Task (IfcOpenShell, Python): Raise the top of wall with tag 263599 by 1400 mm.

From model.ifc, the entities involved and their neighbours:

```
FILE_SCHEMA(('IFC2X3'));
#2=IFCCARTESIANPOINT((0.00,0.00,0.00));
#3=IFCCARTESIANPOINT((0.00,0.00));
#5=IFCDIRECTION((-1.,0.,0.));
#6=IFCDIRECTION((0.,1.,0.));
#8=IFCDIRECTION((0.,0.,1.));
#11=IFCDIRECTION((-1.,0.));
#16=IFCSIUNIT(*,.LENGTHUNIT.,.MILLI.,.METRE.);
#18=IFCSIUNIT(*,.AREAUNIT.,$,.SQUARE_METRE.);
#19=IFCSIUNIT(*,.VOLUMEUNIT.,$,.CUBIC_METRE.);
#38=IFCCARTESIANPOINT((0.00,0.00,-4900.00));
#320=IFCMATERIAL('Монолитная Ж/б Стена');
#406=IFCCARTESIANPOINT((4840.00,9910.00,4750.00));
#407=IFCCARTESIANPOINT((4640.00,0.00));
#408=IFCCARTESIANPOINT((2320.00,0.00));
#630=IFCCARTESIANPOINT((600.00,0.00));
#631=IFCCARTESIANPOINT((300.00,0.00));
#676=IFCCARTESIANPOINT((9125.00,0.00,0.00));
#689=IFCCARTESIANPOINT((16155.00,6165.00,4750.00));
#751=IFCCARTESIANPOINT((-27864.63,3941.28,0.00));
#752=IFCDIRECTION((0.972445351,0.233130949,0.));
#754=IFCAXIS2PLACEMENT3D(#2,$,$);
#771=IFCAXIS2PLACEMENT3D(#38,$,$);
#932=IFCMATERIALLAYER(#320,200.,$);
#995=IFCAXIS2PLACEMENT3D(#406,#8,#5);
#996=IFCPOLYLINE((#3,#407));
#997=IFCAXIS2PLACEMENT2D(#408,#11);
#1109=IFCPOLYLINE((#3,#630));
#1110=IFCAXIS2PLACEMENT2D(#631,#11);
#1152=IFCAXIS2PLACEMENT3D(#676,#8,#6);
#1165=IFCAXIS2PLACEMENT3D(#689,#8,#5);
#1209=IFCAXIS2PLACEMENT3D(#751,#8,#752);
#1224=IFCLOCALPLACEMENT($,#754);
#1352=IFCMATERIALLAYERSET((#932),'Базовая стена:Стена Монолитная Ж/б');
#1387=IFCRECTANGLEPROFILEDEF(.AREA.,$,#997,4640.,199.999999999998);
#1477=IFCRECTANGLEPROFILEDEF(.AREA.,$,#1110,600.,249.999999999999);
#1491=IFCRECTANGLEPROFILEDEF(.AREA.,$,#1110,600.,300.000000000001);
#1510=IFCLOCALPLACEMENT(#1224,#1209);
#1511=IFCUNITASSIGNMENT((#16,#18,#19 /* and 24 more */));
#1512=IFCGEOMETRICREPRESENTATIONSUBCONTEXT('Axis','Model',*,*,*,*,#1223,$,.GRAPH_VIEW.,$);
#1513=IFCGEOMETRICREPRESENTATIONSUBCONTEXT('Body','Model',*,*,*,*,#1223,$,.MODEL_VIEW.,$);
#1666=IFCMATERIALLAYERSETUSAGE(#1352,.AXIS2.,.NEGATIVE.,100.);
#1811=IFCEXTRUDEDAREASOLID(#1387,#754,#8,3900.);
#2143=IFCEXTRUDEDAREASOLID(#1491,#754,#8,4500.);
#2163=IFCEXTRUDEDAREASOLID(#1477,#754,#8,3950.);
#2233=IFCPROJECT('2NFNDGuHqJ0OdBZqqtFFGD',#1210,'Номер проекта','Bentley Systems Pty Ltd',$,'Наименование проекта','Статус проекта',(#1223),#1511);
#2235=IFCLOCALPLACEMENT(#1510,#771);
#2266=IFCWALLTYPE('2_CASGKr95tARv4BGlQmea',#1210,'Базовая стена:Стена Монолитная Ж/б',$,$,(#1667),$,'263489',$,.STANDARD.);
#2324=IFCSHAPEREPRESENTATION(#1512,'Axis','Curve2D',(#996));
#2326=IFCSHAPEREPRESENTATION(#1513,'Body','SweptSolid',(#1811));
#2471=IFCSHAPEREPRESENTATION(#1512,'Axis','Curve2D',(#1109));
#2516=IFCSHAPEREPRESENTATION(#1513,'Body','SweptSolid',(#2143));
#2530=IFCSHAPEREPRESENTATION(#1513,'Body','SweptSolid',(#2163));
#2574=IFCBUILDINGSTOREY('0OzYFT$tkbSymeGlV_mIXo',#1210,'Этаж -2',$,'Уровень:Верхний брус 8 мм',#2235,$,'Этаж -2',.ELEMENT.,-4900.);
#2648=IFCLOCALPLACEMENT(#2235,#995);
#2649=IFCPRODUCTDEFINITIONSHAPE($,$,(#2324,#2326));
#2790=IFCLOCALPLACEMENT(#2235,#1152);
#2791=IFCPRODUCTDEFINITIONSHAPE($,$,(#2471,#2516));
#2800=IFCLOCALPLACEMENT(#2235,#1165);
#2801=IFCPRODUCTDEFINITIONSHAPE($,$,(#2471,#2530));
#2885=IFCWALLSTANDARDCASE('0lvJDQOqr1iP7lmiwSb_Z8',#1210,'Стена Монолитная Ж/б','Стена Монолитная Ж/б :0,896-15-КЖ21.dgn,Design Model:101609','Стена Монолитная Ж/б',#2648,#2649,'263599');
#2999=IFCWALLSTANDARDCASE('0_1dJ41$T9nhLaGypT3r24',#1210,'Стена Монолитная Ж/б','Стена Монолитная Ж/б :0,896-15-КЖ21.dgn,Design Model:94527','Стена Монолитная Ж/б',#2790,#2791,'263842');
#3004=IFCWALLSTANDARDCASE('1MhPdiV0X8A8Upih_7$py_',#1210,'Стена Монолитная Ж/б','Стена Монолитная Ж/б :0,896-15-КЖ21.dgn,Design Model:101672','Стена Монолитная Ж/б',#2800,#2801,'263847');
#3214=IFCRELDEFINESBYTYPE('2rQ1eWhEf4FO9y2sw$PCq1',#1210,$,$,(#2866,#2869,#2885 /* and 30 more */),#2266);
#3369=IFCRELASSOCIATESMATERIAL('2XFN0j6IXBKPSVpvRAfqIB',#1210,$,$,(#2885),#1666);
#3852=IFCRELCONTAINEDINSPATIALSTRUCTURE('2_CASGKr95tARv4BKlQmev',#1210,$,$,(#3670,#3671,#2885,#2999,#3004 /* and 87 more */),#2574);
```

```python
import ifcopenshell
import ifcopenshell.geom
import ifcopenshell.util.representation
import ifcopenshell.util.shape
import ifcopenshell.util.unit

model = ifcopenshell.open("model.ifc")
unit_scale = ifcopenshell.util.unit.calculate_unit_scale(model)
settings = ifcopenshell.geom.settings()


def volume(element):
    """Net volume in cubic metres, openings subtracted."""
    shape = ifcopenshell.geom.create_shape(settings, element)
    return ifcopenshell.util.shape.get_volume(shape.geometry)


wall = model.by_id(2885)
before = volume(wall)

body = ifcopenshell.util.representation.get_representation(wall, "Model", "Body")
solid = body.Items[0]
old_height = solid.Depth
solid.Depth += 1.4 / unit_scale
after = volume(wall)

print(f"height {old_height:g} -> {solid.Depth:g}, volume {before:.3f} -> {after:.3f} m3")

model.write("model_rev.ifc")
```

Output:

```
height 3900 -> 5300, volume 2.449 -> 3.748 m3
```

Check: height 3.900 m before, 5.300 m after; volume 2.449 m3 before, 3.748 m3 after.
